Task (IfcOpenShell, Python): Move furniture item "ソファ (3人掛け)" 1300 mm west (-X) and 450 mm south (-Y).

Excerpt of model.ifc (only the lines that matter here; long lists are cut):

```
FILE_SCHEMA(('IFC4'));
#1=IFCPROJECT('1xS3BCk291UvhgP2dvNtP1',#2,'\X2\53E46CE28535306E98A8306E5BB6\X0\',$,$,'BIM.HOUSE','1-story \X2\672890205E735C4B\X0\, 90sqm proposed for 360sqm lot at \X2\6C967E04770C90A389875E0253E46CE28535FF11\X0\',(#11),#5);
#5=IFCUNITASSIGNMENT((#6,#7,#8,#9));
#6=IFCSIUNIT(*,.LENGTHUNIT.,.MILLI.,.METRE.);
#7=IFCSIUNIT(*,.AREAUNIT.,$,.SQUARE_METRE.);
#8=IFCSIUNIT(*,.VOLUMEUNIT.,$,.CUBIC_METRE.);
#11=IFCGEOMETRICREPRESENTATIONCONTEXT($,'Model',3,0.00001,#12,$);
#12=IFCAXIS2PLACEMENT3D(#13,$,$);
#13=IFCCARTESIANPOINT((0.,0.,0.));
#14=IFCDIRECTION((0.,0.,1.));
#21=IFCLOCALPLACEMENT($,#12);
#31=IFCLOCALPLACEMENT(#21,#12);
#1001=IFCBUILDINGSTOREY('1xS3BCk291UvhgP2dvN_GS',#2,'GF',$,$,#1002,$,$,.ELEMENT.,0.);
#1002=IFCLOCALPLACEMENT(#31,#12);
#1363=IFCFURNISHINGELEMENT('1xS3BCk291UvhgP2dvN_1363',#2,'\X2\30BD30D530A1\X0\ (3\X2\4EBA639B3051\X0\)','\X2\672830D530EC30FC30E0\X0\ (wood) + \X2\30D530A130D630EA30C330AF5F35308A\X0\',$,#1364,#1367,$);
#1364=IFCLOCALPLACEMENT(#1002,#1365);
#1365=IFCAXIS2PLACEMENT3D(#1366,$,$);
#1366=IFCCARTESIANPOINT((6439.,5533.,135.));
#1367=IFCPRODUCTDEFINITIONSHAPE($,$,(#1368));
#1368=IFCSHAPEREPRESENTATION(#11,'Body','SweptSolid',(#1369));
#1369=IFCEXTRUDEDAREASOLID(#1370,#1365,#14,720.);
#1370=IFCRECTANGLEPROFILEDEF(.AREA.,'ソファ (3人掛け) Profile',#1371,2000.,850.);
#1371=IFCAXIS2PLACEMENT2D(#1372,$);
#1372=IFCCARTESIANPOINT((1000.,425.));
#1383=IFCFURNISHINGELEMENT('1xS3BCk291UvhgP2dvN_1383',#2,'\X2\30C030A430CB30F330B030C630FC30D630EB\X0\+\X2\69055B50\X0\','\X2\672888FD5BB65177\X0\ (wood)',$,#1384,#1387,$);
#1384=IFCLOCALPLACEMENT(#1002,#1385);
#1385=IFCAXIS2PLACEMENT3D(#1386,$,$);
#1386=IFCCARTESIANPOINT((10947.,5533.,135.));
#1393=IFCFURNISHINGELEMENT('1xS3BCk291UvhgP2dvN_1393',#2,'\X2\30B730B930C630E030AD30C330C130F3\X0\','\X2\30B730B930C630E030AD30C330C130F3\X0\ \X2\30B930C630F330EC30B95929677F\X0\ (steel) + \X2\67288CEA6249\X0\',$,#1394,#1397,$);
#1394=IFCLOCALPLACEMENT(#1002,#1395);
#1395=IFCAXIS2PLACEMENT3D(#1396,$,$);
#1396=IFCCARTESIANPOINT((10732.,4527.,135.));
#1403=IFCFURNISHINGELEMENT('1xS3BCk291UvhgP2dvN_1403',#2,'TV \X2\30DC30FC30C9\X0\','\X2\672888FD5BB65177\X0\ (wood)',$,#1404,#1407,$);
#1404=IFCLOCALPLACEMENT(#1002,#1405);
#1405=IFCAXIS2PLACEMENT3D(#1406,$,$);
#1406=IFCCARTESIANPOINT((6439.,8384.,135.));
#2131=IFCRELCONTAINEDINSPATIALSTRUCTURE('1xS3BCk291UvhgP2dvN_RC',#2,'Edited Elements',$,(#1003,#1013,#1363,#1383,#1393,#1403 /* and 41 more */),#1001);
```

```python
import ifcopenshell
import ifcopenshell.api.geometry
import ifcopenshell.util.placement

model = ifcopenshell.open("model.ifc")

item = model.by_id(1363)
matrix = ifcopenshell.util.placement.get_local_placement(item.ObjectPlacement)
matrix[0, 3] -= 1300.0
matrix[1, 3] -= 450.0
ifcopenshell.api.geometry.edit_object_placement(model, product=item, matrix=matrix, is_si=False)

print(ifcopenshell.util.placement.get_local_placement(item.ObjectPlacement).round(3) + 0.0)

model.write("model_v2.ifc")
```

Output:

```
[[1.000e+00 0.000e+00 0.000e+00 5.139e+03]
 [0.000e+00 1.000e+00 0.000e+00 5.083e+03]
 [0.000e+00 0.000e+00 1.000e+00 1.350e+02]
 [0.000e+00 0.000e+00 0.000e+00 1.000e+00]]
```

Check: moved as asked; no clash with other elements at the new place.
